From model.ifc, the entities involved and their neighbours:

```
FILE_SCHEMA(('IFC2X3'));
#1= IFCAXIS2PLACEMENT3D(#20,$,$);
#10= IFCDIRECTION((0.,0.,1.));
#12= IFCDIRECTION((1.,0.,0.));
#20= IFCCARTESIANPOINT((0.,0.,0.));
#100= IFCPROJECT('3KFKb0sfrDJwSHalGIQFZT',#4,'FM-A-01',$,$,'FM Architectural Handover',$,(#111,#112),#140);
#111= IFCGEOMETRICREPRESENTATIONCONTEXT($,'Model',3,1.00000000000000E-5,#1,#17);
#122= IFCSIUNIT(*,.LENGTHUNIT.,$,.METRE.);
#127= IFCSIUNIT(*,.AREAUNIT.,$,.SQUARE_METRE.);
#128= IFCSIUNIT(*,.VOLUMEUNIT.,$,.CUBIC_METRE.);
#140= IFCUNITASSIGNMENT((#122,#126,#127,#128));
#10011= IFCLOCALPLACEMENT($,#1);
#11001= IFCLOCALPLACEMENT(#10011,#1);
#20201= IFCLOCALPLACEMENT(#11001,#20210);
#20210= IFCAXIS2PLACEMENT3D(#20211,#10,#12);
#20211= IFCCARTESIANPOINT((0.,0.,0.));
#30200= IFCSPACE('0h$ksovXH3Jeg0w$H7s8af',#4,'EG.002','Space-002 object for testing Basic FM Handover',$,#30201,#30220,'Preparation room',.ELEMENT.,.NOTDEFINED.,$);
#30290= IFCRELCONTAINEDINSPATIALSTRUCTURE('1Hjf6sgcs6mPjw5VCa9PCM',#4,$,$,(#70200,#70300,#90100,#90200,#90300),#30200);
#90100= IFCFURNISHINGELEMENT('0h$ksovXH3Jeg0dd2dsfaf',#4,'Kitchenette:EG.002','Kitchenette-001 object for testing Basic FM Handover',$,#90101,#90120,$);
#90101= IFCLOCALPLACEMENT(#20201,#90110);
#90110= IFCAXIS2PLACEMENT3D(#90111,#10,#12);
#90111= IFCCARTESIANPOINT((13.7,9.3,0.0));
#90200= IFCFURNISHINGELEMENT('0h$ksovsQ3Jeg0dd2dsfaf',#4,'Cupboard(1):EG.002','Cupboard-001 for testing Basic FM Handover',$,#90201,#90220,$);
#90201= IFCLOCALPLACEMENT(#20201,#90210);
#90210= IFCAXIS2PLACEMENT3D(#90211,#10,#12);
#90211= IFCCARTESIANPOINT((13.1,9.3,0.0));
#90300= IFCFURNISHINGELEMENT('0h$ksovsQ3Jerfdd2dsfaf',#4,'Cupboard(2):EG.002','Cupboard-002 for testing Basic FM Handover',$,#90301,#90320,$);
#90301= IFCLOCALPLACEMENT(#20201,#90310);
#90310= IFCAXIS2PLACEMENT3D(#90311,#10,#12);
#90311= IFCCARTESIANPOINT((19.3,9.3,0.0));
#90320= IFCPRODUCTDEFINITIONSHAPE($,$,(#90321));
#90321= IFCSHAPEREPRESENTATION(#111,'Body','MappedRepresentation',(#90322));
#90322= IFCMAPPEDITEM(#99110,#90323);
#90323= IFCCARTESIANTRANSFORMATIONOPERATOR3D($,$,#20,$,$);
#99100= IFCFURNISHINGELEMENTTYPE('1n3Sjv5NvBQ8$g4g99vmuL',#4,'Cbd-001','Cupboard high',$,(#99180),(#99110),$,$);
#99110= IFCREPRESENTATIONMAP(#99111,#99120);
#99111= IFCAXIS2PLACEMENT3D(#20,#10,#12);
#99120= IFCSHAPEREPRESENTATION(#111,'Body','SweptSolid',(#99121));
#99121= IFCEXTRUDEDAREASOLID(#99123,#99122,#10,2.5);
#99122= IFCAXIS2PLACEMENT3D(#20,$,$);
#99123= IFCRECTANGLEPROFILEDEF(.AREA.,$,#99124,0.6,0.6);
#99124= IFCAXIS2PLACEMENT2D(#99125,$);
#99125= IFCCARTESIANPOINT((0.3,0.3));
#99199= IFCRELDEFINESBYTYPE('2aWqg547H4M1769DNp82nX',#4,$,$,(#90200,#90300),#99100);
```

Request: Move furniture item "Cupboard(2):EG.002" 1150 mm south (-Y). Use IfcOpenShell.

```python
import ifcopenshell
import ifcopenshell.api.geometry
import ifcopenshell.util.placement
import ifcopenshell.util.unit

model = ifcopenshell.open("model.ifc")
unit_scale = ifcopenshell.util.unit.calculate_unit_scale(model)

item = model.by_guid("0h$ksovsQ3Jerfdd2dsfaf")
matrix = ifcopenshell.util.placement.get_local_placement(item.ObjectPlacement)
matrix[1, 3] -= 1.15 / unit_scale
ifcopenshell.api.geometry.edit_object_placement(model, product=item, matrix=matrix, is_si=False)

print(ifcopenshell.util.placement.get_local_placement(item.ObjectPlacement).round(3) + 0.0)

model.write("model_rev.ifc")
```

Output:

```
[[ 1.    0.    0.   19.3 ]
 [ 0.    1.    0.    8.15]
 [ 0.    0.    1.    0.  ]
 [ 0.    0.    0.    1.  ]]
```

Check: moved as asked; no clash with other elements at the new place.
